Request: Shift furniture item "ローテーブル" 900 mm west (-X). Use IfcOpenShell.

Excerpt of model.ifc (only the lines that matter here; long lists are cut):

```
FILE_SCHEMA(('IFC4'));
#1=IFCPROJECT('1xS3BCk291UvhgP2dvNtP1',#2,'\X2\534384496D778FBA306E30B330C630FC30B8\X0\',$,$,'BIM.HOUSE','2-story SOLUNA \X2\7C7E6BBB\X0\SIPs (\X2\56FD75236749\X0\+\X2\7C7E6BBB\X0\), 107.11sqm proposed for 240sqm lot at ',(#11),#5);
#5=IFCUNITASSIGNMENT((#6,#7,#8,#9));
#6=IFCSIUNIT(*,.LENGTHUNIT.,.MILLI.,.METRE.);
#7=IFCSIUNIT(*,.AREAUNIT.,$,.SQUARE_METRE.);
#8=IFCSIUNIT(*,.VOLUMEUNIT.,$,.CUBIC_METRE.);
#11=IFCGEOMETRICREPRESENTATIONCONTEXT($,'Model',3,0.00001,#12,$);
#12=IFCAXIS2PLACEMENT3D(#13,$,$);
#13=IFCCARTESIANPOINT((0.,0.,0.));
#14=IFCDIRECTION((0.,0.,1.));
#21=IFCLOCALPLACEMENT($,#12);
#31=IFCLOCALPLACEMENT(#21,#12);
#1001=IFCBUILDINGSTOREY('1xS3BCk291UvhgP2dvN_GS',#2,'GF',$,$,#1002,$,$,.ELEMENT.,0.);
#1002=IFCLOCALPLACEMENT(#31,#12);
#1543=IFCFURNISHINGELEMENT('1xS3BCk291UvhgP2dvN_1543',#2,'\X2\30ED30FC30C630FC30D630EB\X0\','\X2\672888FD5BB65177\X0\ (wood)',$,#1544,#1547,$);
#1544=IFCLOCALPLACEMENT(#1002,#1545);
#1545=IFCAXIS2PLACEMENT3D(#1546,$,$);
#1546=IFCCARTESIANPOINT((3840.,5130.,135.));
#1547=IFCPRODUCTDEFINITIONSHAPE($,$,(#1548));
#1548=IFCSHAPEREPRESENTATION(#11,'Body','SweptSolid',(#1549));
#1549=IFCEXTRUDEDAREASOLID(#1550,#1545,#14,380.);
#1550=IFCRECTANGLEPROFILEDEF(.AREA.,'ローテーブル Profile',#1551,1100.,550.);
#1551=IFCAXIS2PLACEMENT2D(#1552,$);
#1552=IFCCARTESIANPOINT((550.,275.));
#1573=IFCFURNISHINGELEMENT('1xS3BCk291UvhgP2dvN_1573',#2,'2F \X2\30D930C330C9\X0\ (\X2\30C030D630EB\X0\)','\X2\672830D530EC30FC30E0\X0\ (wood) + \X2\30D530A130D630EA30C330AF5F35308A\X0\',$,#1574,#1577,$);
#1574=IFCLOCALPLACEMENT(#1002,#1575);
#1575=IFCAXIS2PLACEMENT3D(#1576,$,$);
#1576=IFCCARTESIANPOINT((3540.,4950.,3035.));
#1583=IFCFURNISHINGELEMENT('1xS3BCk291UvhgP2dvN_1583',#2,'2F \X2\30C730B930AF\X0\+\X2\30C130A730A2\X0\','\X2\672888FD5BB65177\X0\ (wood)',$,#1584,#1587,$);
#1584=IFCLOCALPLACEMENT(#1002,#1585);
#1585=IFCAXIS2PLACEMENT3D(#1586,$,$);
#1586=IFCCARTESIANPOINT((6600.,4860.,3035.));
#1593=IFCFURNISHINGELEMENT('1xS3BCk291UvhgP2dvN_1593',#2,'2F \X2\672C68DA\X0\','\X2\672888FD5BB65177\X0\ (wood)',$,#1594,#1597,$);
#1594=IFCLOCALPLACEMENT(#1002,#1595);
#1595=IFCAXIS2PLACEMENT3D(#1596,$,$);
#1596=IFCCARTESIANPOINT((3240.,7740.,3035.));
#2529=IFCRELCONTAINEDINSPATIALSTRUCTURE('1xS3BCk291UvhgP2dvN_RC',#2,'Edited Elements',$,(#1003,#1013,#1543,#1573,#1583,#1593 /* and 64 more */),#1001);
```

```python
import ifcopenshell
import ifcopenshell.api.geometry
import ifcopenshell.util.placement

model = ifcopenshell.open("model.ifc")

item = model.by_guid("1xS3BCk291UvhgP2dvN_1543")
matrix = ifcopenshell.util.placement.get_local_placement(item.ObjectPlacement)
matrix[0, 3] -= 900.0
ifcopenshell.api.geometry.edit_object_placement(model, product=item, matrix=matrix, is_si=False)

print(ifcopenshell.util.placement.get_local_placement(item.ObjectPlacement).round(3) + 0.0)

model.write("model-out.ifc")
```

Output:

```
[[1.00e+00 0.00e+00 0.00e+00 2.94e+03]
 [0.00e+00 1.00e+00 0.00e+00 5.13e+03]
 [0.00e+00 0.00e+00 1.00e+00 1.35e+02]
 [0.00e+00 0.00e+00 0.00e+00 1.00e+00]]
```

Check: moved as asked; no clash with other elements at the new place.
